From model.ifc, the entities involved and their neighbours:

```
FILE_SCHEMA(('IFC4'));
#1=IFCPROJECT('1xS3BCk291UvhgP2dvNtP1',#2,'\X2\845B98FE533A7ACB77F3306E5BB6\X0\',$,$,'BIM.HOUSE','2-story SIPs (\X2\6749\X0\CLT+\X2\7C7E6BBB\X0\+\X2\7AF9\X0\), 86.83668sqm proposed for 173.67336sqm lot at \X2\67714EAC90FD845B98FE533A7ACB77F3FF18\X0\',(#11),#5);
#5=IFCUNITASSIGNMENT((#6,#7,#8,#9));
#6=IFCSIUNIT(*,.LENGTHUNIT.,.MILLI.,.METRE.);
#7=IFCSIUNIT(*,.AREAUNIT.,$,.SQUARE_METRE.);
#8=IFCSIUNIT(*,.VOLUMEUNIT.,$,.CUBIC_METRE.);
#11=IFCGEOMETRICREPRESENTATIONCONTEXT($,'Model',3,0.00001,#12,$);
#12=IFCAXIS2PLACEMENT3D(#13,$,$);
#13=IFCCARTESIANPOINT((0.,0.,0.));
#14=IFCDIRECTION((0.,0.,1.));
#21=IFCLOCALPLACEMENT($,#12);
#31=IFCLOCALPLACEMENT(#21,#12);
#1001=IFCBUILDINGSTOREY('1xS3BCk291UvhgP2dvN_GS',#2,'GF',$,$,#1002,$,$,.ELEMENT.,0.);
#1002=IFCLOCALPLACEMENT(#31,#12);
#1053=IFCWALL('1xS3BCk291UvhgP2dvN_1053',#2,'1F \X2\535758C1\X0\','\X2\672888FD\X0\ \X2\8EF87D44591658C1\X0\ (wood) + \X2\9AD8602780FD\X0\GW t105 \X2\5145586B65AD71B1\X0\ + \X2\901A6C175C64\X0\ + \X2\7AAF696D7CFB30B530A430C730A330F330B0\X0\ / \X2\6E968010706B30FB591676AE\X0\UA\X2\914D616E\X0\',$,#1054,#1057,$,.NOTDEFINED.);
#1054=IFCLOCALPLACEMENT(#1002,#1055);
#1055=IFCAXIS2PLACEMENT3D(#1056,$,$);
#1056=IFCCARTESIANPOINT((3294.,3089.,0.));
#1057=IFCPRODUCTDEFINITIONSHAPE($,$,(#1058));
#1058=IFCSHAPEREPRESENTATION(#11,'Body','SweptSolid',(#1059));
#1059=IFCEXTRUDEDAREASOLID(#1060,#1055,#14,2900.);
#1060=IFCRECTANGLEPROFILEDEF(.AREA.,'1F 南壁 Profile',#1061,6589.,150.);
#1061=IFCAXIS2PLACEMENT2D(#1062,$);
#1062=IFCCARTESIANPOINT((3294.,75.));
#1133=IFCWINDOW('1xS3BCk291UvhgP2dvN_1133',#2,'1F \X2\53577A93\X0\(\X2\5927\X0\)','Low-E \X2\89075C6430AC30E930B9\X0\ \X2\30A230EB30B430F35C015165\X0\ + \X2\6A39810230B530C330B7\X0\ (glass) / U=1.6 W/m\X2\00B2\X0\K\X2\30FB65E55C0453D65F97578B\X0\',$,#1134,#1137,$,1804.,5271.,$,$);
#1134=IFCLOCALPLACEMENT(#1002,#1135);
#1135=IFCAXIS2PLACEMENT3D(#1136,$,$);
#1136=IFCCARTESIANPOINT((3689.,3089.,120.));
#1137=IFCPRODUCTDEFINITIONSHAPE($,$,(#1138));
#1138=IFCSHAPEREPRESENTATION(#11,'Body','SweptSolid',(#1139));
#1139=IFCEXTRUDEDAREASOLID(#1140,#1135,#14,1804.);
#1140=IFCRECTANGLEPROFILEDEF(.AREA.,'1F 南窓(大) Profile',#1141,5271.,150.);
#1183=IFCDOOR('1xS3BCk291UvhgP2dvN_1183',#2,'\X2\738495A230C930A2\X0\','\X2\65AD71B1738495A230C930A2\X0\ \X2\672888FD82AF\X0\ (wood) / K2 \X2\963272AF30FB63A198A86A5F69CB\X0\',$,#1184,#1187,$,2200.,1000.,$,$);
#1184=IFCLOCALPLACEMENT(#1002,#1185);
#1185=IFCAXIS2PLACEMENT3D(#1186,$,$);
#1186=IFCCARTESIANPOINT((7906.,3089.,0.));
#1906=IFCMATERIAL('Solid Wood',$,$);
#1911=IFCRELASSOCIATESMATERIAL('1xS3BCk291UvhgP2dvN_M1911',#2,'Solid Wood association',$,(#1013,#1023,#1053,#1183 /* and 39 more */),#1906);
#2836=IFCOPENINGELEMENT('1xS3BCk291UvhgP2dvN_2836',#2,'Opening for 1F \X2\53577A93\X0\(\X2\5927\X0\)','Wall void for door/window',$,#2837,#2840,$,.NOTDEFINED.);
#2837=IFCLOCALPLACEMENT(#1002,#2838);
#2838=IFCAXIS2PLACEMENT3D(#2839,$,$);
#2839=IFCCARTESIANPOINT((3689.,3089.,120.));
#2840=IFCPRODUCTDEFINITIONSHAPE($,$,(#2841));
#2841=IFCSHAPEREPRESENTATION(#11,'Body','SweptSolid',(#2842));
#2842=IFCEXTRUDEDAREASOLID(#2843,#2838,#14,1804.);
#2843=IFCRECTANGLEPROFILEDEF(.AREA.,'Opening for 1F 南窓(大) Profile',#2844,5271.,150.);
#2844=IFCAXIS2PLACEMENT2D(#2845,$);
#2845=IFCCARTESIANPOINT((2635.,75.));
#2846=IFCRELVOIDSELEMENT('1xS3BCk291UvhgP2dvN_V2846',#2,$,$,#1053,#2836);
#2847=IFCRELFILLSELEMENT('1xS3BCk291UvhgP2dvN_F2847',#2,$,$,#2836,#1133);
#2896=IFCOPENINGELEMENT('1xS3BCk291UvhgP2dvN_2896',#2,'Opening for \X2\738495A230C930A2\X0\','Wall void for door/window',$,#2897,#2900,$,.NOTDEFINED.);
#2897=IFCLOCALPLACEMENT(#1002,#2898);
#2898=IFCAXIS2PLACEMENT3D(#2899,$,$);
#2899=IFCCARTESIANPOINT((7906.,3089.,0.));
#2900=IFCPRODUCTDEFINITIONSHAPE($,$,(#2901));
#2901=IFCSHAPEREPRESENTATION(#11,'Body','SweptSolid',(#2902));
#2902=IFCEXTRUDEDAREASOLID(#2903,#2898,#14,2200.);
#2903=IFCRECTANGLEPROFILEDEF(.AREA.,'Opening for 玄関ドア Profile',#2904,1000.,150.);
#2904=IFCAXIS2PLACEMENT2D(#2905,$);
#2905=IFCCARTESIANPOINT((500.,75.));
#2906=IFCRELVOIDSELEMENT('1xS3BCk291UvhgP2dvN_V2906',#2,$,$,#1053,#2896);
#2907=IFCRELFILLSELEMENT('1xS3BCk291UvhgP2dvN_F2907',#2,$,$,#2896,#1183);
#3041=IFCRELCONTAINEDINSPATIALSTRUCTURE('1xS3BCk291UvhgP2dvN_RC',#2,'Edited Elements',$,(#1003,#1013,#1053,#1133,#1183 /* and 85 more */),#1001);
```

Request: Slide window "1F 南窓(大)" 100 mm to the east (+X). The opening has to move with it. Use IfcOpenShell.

```python
import ifcopenshell
import ifcopenshell.api.geometry
import ifcopenshell.util.placement

model = ifcopenshell.open("model.ifc")

window = model.by_guid("1xS3BCk291UvhgP2dvN_1133")
opening = window.FillsVoids[0].RelatingOpeningElement
wall = opening.VoidsElements[0].RelatingBuildingElement

wall_matrix = ifcopenshell.util.placement.get_local_placement(wall.ObjectPlacement)
shift = wall_matrix[:3, 0] * 100.0
before = ifcopenshell.util.placement.get_local_placement(window.ObjectPlacement)[:3, 3].copy()

# The window is not placed relative to its opening, so move both.
for product in (opening, window):
    matrix = ifcopenshell.util.placement.get_local_placement(product.ObjectPlacement)
    matrix[:3, 3] += shift
    ifcopenshell.api.geometry.edit_object_placement(model, product=product, matrix=matrix, is_si=False)

after = ifcopenshell.util.placement.get_local_placement(window.ObjectPlacement)[:3, 3]
print("window moved by", (after - before).round(3) + 0.0)

model.write("model_edited.ifc")
```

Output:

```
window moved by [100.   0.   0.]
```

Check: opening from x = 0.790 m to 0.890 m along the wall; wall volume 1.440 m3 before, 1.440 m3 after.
